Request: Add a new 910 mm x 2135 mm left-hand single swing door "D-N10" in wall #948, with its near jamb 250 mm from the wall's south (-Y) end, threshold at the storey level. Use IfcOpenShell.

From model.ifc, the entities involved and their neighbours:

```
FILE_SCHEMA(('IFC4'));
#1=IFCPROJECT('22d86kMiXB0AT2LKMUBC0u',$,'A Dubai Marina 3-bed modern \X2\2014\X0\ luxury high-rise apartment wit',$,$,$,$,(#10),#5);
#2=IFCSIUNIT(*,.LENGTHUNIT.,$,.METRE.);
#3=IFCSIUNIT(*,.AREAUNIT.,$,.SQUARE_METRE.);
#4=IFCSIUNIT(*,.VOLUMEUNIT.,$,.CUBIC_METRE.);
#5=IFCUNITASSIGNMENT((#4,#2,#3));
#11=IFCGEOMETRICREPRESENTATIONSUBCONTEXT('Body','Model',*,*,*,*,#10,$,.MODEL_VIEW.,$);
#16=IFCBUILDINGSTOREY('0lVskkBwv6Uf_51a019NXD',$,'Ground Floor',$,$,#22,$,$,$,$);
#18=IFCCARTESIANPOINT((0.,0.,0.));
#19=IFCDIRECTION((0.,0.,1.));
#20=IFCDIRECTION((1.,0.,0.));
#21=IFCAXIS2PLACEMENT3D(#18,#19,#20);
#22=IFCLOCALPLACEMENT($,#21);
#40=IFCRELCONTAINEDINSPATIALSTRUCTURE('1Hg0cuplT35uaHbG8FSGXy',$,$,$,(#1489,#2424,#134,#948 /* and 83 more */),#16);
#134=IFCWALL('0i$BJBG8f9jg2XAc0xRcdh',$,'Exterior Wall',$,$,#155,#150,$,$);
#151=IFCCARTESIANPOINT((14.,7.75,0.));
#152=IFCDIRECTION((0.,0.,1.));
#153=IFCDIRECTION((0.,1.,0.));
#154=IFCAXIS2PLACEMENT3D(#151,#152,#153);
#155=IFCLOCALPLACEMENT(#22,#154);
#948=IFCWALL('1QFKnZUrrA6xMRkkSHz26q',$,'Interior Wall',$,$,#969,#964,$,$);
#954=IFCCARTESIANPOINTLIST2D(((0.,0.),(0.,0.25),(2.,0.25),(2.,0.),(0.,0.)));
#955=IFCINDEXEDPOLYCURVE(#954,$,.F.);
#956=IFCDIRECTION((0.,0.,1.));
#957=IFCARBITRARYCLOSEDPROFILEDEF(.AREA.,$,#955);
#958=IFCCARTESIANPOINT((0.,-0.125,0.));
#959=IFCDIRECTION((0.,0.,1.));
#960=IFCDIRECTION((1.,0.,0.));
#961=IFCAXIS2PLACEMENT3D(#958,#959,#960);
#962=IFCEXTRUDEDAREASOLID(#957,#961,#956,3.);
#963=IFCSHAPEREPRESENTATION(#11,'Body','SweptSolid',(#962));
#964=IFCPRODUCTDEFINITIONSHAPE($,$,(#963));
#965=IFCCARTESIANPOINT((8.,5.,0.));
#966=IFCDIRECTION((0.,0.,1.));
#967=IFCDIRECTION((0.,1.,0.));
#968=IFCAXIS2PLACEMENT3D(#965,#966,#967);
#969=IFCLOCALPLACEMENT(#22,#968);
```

```python
import numpy as np
import ifcopenshell
import ifcopenshell.api.feature
import ifcopenshell.api.geometry
import ifcopenshell.api.root
import ifcopenshell.api.spatial
import ifcopenshell.geom
import ifcopenshell.util.element
import ifcopenshell.util.placement
import ifcopenshell.util.representation
import ifcopenshell.util.shape
import ifcopenshell.util.unit

model = ifcopenshell.open("model.ifc")
unit_scale = ifcopenshell.util.unit.calculate_unit_scale(model)
settings = ifcopenshell.geom.settings()


def volume(element):
    """Net volume in cubic metres, openings subtracted."""
    shape = ifcopenshell.geom.create_shape(settings, element)
    return ifcopenshell.util.shape.get_volume(shape.geometry)


wall = model.by_guid("1QFKnZUrrA6xMRkkSHz26q")
storey = ifcopenshell.util.element.get_container(wall, ifc_class="IfcBuildingStorey")
context = ifcopenshell.util.representation.get_context(model, "Model", "Body", "MODEL_VIEW")
before = volume(wall)

width, height, from_end, sill = 0.91, 2.135, 0.25, 0.0  # metres

# The wall runs along its own X axis, and the end named is its -X end.
wall_shape = ifcopenshell.geom.create_shape(settings, wall)
x, y, z = ifcopenshell.util.shape.get_vertices(wall_shape.geometry).T
start = x.min() + from_end
face, thickness = float(y.min()), float(y.max() - y.min())
wall_matrix = ifcopenshell.util.placement.get_local_placement(wall.ObjectPlacement)
level = ifcopenshell.util.placement.get_local_placement(storey.ObjectPlacement)[2, 3]


def in_wall(x, y):
    """Placement at x, y metres in the wall's axes, at sill height."""
    matrix = wall_matrix.copy()
    matrix[:, 3] = wall_matrix @ np.array([x / unit_scale, y / unit_scale, 0.0, 1.0])
    matrix[2, 3] = level + sill / unit_scale
    return matrix


# Opening: a box that overshoots both wall faces by 50 mm.
opening = ifcopenshell.api.root.create_entity(model, ifc_class="IfcOpeningElement", predefined_type="OPENING")
box = ifcopenshell.api.geometry.add_wall_representation(
    model, context=context, length=width, height=height, thickness=thickness + 0.1
)
ifcopenshell.api.geometry.assign_representation(model, product=opening, representation=box)
ifcopenshell.api.geometry.edit_object_placement(model, product=opening, matrix=in_wall(start, face - 0.05), is_si=False)
ifcopenshell.api.feature.add_feature(model, feature=opening, element=wall)

door = ifcopenshell.api.root.create_entity(model, ifc_class="IfcDoor", name="D-N10", predefined_type="DOOR")
door.OverallWidth, door.OverallHeight = width / unit_scale, height / unit_scale
door.OperationType = "SINGLE_SWING_LEFT"
body = ifcopenshell.api.geometry.add_door_representation(
    model,
    context=context,
    overall_width=door.OverallWidth,
    overall_height=door.OverallHeight,
    operation_type="SINGLE_SWING_LEFT",
    lining_properties={"LiningDepth": thickness / unit_scale, "ThresholdDepth": thickness / unit_scale},
)
ifcopenshell.api.geometry.assign_representation(model, product=door, representation=body)
ifcopenshell.api.spatial.assign_container(model, products=[door], relating_structure=storey)
ifcopenshell.api.feature.add_filling(model, opening=opening, element=door)

# The lining spans the wall, so the door starts at the wall face.
ifcopenshell.api.geometry.edit_object_placement(model, product=door, matrix=in_wall(start, face), is_si=False)

after = volume(wall)

print(f"wall volume {before:.3f} -> {after:.3f} m3")

model.write("model_edited.ifc")
```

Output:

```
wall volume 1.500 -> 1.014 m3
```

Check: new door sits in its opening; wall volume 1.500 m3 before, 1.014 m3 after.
